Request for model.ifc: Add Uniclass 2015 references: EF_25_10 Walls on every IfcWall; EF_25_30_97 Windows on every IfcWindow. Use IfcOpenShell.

First a look at what the model holds.

```python
import ifcopenshell

model = ifcopenshell.open("model.ifc")
print(model.schema)
print("classifications:", [c.Name for c in model.by_type("IfcClassification")])
for ifc_class in ("IfcDoor", "IfcRoof", "IfcStair", "IfcWall", "IfcWindow"):
    print(ifc_class, len(model.by_type(ifc_class)))
```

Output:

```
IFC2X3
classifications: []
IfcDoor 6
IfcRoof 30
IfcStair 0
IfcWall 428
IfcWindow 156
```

```python
import ifcopenshell
import ifcopenshell.api.classification

model = ifcopenshell.open("model.ifc")

# IFC2X3 requires Source and Edition and has no link from the project to the system.
system = model.create_entity("IfcClassification", Source="NBS", Edition="2015", Name="Uniclass 2015")

codes = {
    "IfcWall": ("EF_25_10", "Walls"),
    "IfcWindow": ("EF_25_30_97", "Windows"),
}
for ifc_class, (code, name) in codes.items():
    products = model.by_type(ifc_class)
    ifcopenshell.api.classification.add_reference(
        model, products=products, classification=system, identification=code, name=name
    )
    print(code, len(products))

model.write("model-out.ifc")
```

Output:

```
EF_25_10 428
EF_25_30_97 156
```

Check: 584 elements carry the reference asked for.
